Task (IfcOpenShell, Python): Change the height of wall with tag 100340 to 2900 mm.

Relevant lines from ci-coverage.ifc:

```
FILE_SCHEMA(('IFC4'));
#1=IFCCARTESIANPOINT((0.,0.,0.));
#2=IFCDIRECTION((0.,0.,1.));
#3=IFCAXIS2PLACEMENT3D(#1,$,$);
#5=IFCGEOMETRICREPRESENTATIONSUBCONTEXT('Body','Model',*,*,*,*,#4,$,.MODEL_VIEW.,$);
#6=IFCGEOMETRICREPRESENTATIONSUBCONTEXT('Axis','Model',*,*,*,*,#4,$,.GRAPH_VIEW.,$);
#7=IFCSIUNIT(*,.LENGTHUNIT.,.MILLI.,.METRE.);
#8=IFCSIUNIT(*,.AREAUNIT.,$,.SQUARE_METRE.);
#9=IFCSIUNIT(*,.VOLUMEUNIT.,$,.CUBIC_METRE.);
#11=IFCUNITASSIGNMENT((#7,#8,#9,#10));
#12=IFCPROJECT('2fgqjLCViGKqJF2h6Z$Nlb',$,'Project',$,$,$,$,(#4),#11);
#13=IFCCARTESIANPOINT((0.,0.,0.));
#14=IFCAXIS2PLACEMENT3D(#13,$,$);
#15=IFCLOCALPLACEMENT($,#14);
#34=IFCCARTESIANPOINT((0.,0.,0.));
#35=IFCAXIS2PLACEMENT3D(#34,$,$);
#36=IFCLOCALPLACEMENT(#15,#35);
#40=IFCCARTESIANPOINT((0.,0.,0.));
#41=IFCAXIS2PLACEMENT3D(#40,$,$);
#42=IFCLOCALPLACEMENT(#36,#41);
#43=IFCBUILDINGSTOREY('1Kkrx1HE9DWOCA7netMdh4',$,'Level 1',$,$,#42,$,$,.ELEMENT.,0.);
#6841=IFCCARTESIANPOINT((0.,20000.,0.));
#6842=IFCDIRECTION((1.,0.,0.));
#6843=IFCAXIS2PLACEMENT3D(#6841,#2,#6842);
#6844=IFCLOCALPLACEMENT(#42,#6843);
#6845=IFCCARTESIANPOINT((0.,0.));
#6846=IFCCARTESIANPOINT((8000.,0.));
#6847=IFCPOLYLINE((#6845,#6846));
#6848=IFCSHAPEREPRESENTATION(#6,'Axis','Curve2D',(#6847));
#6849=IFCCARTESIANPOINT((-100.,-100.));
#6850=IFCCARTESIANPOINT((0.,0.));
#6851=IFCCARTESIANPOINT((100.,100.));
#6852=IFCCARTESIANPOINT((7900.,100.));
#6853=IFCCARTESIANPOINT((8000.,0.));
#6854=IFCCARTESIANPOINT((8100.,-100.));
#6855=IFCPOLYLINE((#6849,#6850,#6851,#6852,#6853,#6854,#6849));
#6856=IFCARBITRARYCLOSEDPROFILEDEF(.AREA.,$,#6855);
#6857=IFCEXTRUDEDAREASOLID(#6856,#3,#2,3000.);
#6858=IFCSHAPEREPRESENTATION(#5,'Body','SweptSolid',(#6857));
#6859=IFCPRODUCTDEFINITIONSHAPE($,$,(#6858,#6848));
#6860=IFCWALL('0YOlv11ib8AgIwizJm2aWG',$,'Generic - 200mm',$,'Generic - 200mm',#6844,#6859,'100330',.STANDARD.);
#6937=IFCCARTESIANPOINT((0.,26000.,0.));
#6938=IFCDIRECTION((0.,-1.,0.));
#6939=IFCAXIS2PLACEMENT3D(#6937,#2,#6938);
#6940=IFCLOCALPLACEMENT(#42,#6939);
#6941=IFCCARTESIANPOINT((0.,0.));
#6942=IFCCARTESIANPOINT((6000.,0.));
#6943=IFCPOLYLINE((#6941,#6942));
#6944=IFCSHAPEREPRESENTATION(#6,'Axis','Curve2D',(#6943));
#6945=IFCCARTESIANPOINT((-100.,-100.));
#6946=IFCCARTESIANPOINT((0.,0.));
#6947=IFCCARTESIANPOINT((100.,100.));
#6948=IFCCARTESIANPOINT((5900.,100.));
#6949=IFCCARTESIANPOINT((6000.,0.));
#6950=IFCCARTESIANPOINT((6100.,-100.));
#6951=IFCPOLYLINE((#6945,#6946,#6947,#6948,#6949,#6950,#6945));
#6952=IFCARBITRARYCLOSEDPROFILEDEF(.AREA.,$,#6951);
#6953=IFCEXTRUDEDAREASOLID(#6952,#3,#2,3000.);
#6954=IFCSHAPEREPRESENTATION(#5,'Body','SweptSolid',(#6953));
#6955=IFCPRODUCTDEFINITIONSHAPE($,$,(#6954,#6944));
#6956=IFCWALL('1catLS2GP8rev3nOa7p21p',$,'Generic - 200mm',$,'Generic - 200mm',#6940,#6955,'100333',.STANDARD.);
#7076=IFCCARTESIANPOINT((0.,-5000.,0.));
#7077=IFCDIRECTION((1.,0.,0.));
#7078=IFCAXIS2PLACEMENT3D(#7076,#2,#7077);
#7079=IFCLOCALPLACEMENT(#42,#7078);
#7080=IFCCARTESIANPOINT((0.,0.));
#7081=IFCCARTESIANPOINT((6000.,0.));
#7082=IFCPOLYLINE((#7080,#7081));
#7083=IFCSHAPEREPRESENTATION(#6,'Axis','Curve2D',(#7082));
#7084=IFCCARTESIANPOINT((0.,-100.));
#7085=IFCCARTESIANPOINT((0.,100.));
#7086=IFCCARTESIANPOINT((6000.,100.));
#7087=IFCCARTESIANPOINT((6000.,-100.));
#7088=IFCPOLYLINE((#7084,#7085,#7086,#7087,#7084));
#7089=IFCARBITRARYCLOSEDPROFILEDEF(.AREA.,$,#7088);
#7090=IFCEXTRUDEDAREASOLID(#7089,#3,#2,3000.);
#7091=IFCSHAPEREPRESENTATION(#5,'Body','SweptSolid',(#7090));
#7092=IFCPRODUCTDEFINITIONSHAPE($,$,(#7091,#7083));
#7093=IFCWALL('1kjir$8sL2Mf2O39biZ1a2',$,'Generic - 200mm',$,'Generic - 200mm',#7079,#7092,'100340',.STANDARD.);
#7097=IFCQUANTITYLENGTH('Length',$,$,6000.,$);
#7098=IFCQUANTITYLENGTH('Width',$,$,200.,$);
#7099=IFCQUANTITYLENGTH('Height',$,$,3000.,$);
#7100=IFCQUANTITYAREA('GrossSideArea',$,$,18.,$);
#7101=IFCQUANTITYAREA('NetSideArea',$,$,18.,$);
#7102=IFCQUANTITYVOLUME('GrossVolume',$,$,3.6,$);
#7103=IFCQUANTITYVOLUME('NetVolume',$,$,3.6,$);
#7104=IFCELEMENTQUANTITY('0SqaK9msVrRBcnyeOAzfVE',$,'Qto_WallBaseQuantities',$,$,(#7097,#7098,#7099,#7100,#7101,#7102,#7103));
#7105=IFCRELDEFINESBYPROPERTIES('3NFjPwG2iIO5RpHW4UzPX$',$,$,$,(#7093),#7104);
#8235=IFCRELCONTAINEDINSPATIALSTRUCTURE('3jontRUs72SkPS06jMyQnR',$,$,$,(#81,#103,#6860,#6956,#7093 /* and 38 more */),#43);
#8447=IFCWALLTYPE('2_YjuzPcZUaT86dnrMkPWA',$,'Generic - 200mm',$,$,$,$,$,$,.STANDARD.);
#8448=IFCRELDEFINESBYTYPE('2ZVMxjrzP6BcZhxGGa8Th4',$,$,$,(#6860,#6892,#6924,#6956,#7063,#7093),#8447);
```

```python
import ifcopenshell
import ifcopenshell.api.pset
import ifcopenshell.geom
import ifcopenshell.util.element
import ifcopenshell.util.representation
import ifcopenshell.util.shape
import ifcopenshell.util.unit

model = ifcopenshell.open("ci-coverage.ifc")
unit_scale = ifcopenshell.util.unit.calculate_unit_scale(model)
area_scale = ifcopenshell.util.unit.calculate_unit_scale(model, "AREAUNIT")
volume_scale = ifcopenshell.util.unit.calculate_unit_scale(model, "VOLUMEUNIT")
settings = ifcopenshell.geom.settings()


def volume(element):
    """Net volume in cubic metres, openings subtracted."""
    shape = ifcopenshell.geom.create_shape(settings, element)
    return ifcopenshell.util.shape.get_volume(shape.geometry)


wall = model.by_guid("1kjir$8sL2Mf2O39biZ1a2")
before = volume(wall)

body = ifcopenshell.util.representation.get_representation(wall, "Model", "Body")
solid = body.Items[0]
old_height = solid.Depth
solid.Depth = 2.9 / unit_scale
after = volume(wall)
thickness = 0.2  # wall thickness in metres

# Update the stored height, areas and volumes.
qto = model.by_id(ifcopenshell.util.element.get_pset(wall, "Qto_WallBaseQuantities", should_inherit=False)["id"])
ifcopenshell.api.pset.edit_qto(model, qto=qto, properties={
    "Height": solid.Depth,
    "GrossSideArea": ifcopenshell.util.element.get_pset(wall, "Qto_WallBaseQuantities", "GrossSideArea") * solid.Depth / old_height,
    "NetSideArea": after / thickness / area_scale,
    "GrossVolume": ifcopenshell.util.element.get_pset(wall, "Qto_WallBaseQuantities", "GrossVolume") * solid.Depth / old_height,
    "NetVolume": after / volume_scale,
})

print(f"height {old_height:g} -> {solid.Depth:g}, volume {before:.3f} -> {after:.3f} m3")

model.write("ci-coverage_updated.ifc")
```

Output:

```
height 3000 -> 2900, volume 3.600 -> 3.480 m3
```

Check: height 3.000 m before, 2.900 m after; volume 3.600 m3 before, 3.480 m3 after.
